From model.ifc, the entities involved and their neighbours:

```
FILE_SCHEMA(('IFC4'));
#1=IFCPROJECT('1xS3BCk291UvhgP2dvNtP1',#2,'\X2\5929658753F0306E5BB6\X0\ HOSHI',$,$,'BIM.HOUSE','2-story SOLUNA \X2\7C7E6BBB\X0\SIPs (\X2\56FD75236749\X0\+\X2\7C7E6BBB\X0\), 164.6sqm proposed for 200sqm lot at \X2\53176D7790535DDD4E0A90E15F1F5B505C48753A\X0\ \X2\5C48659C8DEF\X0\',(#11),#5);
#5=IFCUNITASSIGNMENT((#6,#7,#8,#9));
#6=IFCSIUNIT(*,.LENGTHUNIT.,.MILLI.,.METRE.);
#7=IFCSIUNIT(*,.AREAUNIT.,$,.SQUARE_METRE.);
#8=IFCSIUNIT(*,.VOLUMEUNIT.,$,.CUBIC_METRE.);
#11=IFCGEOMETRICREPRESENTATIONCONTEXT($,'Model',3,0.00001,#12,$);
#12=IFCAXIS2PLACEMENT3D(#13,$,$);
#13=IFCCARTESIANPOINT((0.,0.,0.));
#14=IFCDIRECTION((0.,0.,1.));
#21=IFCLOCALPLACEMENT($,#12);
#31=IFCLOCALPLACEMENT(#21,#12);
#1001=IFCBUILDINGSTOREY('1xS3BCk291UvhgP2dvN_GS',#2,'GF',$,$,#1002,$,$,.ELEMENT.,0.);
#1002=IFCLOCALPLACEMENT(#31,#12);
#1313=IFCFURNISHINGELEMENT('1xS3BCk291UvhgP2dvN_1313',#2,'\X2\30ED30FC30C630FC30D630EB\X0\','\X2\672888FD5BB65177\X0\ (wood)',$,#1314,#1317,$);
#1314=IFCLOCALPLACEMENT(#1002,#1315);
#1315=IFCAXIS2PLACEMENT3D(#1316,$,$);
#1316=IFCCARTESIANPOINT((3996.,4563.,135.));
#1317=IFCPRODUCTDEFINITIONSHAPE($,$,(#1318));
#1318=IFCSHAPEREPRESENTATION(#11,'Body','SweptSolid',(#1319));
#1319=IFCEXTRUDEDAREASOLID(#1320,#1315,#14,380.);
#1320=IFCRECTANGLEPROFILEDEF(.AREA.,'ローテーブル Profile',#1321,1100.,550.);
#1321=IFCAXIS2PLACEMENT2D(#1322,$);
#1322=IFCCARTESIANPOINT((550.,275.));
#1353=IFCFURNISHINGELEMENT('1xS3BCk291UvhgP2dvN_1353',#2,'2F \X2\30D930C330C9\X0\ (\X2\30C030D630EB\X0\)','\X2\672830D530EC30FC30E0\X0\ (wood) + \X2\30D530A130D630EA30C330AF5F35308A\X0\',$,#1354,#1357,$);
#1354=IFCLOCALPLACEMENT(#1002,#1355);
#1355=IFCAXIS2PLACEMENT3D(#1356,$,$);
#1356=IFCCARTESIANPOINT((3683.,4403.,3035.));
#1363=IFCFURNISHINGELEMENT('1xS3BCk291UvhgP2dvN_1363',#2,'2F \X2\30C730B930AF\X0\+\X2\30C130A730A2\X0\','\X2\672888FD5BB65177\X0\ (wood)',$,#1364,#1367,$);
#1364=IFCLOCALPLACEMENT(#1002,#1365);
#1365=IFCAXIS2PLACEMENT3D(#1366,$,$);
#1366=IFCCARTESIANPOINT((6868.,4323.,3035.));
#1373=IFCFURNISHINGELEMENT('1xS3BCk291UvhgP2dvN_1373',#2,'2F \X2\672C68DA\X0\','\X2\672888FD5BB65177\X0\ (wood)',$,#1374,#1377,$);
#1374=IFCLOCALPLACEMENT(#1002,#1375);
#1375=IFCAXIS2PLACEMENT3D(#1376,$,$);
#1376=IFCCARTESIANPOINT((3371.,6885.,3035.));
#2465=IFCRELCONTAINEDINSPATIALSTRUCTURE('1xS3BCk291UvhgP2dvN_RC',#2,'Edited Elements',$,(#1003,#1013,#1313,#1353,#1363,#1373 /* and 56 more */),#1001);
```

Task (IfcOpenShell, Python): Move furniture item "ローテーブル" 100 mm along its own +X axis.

```python
import ifcopenshell
import ifcopenshell.api.geometry
import ifcopenshell.util.placement
import ifcopenshell.util.unit

model = ifcopenshell.open("model.ifc")
unit_scale = ifcopenshell.util.unit.calculate_unit_scale(model)

item = model.by_guid("1xS3BCk291UvhgP2dvN_1313")
matrix = ifcopenshell.util.placement.get_local_placement(item.ObjectPlacement)
matrix[:3, 3] += matrix[:3, 0] * 0.1 / unit_scale
ifcopenshell.api.geometry.edit_object_placement(model, product=item, matrix=matrix, is_si=False)

print(ifcopenshell.util.placement.get_local_placement(item.ObjectPlacement).round(3) + 0.0)

model.write("model-out.ifc")
```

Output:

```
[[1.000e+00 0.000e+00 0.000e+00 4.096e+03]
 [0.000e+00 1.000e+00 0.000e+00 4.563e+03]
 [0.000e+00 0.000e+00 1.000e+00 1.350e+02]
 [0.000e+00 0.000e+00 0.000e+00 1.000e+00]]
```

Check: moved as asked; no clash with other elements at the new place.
